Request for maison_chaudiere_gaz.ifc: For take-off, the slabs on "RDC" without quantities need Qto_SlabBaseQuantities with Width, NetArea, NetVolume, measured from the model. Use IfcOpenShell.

First a look at what the model holds.

```python
import ifcopenshell
import ifcopenshell.util.element
import ifcopenshell.util.unit

model = ifcopenshell.open("maison_chaudiere_gaz.ifc")
print(model.schema)
for unit_type in ("LENGTHUNIT", "AREAUNIT", "VOLUMEUNIT"):
    print(unit_type, ifcopenshell.util.unit.calculate_unit_scale(model, unit_type))
storey = next(s for s in model.by_type("IfcBuildingStorey") if s.Name == "RDC")
slabs = [e for e in ifcopenshell.util.element.get_decomposition(storey) if e.is_a("IfcSlab")]
for e in sorted(slabs, key=lambda e: e.id()):
    print(e.id(), e.is_a(), e.Name, list(ifcopenshell.util.element.get_psets(e, qtos_only=True)), sep=" | ")
```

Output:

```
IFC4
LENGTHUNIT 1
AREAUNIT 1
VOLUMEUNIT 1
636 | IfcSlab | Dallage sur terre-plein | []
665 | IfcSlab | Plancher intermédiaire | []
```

```python
import ifcopenshell
import ifcopenshell.api.pset
import ifcopenshell.geom
import ifcopenshell.util.element
import ifcopenshell.util.shape
import ifcopenshell.util.unit

model = ifcopenshell.open("maison_chaudiere_gaz.ifc")
unit_scale = ifcopenshell.util.unit.calculate_unit_scale(model)
area_scale = ifcopenshell.util.unit.calculate_unit_scale(model, "AREAUNIT")
volume_scale = ifcopenshell.util.unit.calculate_unit_scale(model, "VOLUMEUNIT")
settings = ifcopenshell.geom.settings()

storey = next(s for s in model.by_type("IfcBuildingStorey") if s.Name == "RDC")
slabs = [e for e in ifcopenshell.util.element.get_decomposition(storey) if e.is_a("IfcSlab")]

for e in sorted(slabs, key=lambda e: e.id()):
    if ifcopenshell.util.element.get_psets(e, qtos_only=True, should_inherit=False):
        continue
    # Geometry comes back in metres, in the element's own axes.
    shape = ifcopenshell.geom.create_shape(settings, e)
    values = {
        "Width": ifcopenshell.util.shape.get_z(shape.geometry) / unit_scale,
        "NetArea": ifcopenshell.util.shape.get_footprint_area(shape.geometry) / area_scale,
        "NetVolume": ifcopenshell.util.shape.get_volume(shape.geometry) / volume_scale,
    }
    qto = ifcopenshell.api.pset.add_qto(model, product=e, name="Qto_SlabBaseQuantities")
    ifcopenshell.api.pset.edit_qto(model, qto=qto, properties=values)
    print(e.id(), {k: round(v, 3) for k, v in values.items()})

model.write("maison_chaudiere_gaz_updated.ifc")
```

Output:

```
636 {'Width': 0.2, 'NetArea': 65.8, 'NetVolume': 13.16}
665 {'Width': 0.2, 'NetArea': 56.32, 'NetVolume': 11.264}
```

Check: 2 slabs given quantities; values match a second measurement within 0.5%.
